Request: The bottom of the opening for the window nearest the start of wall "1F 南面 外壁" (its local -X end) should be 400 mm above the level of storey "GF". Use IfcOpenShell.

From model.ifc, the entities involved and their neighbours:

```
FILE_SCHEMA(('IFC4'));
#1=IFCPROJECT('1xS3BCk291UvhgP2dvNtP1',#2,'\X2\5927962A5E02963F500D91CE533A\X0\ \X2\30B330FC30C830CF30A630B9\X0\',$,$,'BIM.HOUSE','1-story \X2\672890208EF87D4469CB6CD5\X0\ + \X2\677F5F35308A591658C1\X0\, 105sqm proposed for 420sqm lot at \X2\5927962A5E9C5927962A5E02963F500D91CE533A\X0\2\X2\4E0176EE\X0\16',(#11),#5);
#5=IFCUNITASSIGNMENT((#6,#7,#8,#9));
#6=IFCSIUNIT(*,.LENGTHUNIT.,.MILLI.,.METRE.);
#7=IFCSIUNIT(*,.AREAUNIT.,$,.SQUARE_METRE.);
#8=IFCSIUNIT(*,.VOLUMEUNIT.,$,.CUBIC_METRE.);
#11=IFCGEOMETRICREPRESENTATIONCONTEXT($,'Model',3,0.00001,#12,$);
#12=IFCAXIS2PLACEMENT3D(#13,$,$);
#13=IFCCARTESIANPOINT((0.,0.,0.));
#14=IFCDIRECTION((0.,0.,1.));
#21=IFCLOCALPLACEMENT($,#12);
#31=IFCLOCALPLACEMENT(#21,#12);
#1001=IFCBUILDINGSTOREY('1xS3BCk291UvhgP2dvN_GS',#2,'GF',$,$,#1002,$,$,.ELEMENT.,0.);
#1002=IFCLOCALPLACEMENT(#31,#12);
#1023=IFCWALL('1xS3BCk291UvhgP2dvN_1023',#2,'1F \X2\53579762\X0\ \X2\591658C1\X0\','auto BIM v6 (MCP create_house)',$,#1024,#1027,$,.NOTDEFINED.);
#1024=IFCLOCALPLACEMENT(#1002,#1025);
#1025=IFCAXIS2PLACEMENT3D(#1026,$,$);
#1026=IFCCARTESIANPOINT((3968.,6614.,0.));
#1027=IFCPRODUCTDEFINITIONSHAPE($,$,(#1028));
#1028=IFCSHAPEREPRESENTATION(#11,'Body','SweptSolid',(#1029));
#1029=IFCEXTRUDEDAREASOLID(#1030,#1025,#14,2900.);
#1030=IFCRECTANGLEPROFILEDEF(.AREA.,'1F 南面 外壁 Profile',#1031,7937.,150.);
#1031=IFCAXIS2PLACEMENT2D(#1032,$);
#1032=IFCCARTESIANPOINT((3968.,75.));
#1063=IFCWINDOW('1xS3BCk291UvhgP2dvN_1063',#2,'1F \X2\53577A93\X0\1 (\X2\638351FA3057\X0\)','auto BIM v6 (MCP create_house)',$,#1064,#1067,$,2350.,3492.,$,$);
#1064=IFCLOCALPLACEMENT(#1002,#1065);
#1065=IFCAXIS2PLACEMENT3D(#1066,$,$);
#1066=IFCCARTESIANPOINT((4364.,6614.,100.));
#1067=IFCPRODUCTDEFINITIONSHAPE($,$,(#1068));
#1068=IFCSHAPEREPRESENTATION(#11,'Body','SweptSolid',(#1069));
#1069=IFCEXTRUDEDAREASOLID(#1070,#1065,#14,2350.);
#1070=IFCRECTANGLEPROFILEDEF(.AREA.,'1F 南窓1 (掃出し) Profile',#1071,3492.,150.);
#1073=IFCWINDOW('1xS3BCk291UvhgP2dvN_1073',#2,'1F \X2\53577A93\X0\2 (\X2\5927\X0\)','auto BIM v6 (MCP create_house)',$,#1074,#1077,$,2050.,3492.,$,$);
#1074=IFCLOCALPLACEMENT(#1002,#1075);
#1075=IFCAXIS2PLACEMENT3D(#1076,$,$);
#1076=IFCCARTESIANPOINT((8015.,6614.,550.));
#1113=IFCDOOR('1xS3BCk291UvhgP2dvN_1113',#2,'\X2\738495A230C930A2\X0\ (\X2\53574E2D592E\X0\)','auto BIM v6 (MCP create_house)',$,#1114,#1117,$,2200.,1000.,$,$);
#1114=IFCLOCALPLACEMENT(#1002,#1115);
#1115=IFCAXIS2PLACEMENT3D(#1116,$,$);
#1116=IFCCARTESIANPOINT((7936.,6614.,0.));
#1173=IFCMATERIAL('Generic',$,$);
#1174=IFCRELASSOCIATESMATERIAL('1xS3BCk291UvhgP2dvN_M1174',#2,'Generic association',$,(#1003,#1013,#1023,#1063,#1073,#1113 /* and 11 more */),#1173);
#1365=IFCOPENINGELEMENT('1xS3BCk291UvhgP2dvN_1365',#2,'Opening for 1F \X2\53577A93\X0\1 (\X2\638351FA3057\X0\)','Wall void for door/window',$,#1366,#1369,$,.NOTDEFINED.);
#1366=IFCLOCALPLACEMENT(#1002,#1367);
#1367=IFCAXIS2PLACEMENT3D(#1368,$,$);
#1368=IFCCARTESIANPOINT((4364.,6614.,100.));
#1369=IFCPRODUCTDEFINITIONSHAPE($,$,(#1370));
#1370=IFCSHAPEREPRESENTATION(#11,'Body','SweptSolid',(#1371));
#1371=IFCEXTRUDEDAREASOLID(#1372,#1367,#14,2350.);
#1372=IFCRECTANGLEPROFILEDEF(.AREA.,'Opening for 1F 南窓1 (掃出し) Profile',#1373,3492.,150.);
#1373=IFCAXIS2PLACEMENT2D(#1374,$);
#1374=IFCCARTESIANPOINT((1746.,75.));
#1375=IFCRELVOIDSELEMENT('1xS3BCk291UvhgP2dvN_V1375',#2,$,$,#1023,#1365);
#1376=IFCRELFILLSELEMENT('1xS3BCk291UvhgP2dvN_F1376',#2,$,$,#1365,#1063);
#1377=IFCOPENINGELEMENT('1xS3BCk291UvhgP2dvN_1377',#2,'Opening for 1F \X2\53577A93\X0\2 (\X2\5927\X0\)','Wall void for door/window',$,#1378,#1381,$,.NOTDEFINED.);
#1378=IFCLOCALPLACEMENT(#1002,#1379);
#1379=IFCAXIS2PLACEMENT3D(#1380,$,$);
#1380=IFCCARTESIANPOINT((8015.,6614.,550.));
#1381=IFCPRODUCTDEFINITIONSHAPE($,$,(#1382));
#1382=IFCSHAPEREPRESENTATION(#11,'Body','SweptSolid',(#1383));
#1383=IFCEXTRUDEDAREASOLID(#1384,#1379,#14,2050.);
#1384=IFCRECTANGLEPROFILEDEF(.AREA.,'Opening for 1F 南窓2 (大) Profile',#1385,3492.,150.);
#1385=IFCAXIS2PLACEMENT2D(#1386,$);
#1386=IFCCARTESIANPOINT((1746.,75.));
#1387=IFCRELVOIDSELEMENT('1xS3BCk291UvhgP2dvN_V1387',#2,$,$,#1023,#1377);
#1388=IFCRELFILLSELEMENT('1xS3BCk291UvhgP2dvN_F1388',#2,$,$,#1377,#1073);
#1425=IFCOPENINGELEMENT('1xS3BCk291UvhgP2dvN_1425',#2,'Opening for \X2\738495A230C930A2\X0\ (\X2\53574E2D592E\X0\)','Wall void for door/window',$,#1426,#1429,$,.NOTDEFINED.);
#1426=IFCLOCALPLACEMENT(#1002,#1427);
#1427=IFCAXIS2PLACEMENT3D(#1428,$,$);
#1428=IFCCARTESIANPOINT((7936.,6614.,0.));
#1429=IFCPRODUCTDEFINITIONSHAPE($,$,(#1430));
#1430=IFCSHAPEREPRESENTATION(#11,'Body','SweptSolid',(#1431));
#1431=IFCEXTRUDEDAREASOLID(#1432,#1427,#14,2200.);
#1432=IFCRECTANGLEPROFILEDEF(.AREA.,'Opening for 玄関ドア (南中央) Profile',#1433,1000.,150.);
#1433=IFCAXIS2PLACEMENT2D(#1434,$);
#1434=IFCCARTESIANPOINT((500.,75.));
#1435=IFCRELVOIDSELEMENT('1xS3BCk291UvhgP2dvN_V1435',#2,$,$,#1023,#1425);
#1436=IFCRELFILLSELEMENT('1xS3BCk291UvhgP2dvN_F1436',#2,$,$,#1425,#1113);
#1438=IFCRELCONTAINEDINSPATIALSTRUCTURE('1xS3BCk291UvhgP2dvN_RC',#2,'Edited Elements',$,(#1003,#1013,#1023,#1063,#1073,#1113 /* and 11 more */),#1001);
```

```python
import numpy as np
import ifcopenshell
import ifcopenshell.api.geometry
import ifcopenshell.geom
import ifcopenshell.util.element
import ifcopenshell.util.placement
import ifcopenshell.util.shape
import ifcopenshell.util.unit

model = ifcopenshell.open("model.ifc")
unit_scale = ifcopenshell.util.unit.calculate_unit_scale(model)

window = model.by_id(1063)
opening = window.FillsVoids[0].RelatingOpeningElement
storey = ifcopenshell.util.element.get_container(window, ifc_class="IfcBuildingStorey")
level = ifcopenshell.util.placement.get_local_placement(storey.ObjectPlacement)[2, 3]

# The opening's origin need not be at the sill, so measure its lowest point.
shape = ifcopenshell.geom.create_shape(ifcopenshell.geom.settings(), opening)
bottom = ifcopenshell.util.shape.get_shape_bottom_elevation(shape, shape.geometry) / unit_scale
dz = level + 0.4 / unit_scale - bottom

shift = np.array([0.0, 0.0, dz])
# The window is not placed relative to its opening, so move both.
for product in (opening, window):
    matrix = ifcopenshell.util.placement.get_local_placement(product.ObjectPlacement)
    matrix[:3, 3] += shift
    ifcopenshell.api.geometry.edit_object_placement(model, product=product, matrix=matrix, is_si=False)

print(f"moved by {dz * unit_scale:+.3f} m")

model.write("model-out.ifc")
```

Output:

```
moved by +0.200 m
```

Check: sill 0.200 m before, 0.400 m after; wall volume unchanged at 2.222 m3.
